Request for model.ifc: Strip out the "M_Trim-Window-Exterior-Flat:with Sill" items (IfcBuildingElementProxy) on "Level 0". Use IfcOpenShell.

First a look at what the model holds.

```python
import ifcopenshell
import ifcopenshell.util.element

model = ifcopenshell.open("model.ifc")
print(model.schema)
storey = next(s for s in model.by_type("IfcBuildingStorey") if s.Name == "Level 0")
proxies = [e for e in ifcopenshell.util.element.get_decomposition(storey) if e.is_a("IfcBuildingElementProxy")]
seen = {}
for e in proxies:
    element_type = ifcopenshell.util.element.get_type(e)
    name = element_type.Name if element_type not in (None, e) else None
    seen[name] = seen.get(name, 0) + 1
for name, count in sorted(seen.items(), key=str):
    print(count, "x", name)
```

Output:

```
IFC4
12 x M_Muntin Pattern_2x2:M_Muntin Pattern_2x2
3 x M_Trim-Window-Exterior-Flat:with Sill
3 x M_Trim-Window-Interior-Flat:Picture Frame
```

```python
import ifcopenshell
import ifcopenshell.api.root
import ifcopenshell.util.element

model = ifcopenshell.open("model.ifc")

storey = next(s for s in model.by_type("IfcBuildingStorey") if s.Name == "Level 0")
proxies = [e for e in ifcopenshell.util.element.get_decomposition(storey) if e.is_a("IfcBuildingElementProxy")]
targets = [e for e in proxies if (t := ifcopenshell.util.element.get_type(e)) not in (None, e) and t.Name == "M_Trim-Window-Exterior-Flat:with Sill"]

for e in targets:
    ifcopenshell.api.root.remove_product(model, product=e)
print(len(targets), "removed")

model.write("model_edited.ifc")
```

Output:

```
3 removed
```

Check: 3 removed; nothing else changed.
